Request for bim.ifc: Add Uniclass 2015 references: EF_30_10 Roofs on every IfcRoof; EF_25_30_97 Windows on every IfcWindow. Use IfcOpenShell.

First a look at what the model holds.

```python
import ifcopenshell

model = ifcopenshell.open("bim.ifc")
print(model.schema)
print("classifications:", [c.Name for c in model.by_type("IfcClassification")])
for ifc_class in ("IfcDoor", "IfcRoof", "IfcStair", "IfcWall", "IfcWindow"):
    print(ifc_class, len(model.by_type(ifc_class)))
```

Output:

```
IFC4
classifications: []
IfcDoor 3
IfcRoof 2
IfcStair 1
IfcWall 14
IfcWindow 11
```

```python
import ifcopenshell
import ifcopenshell.api.classification

model = ifcopenshell.open("bim.ifc")

system = ifcopenshell.api.classification.add_classification(model, classification="Uniclass 2015")

codes = {
    "IfcRoof": ("EF_30_10", "Roofs"),
    "IfcWindow": ("EF_25_30_97", "Windows"),
}
for ifc_class, (code, name) in codes.items():
    products = model.by_type(ifc_class)
    ifcopenshell.api.classification.add_reference(
        model, products=products, classification=system, identification=code, name=name
    )
    print(code, len(products))

model.write("bim-out.ifc")
```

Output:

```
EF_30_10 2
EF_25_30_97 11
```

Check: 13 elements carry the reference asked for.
